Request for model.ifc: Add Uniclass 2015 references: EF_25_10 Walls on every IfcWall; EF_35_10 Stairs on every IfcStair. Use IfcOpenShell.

First a look at what the model holds.

```python
import ifcopenshell

model = ifcopenshell.open("model.ifc")
print(model.schema)
print("classifications:", [c.Name for c in model.by_type("IfcClassification")])
for ifc_class in ("IfcDoor", "IfcRoof", "IfcStair", "IfcWall", "IfcWindow"):
    print(ifc_class, len(model.by_type(ifc_class)))
```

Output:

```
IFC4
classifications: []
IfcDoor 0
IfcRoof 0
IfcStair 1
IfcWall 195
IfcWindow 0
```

```python
import ifcopenshell
import ifcopenshell.api.classification

model = ifcopenshell.open("model.ifc")

system = ifcopenshell.api.classification.add_classification(model, classification="Uniclass 2015")

codes = {
    "IfcWall": ("EF_25_10", "Walls"),
    "IfcStair": ("EF_35_10", "Stairs"),
}
for ifc_class, (code, name) in codes.items():
    products = model.by_type(ifc_class)
    ifcopenshell.api.classification.add_reference(
        model, products=products, classification=system, identification=code, name=name
    )
    print(code, len(products))

model.write("model_edited.ifc")
```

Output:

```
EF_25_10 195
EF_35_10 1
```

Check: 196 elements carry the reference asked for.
